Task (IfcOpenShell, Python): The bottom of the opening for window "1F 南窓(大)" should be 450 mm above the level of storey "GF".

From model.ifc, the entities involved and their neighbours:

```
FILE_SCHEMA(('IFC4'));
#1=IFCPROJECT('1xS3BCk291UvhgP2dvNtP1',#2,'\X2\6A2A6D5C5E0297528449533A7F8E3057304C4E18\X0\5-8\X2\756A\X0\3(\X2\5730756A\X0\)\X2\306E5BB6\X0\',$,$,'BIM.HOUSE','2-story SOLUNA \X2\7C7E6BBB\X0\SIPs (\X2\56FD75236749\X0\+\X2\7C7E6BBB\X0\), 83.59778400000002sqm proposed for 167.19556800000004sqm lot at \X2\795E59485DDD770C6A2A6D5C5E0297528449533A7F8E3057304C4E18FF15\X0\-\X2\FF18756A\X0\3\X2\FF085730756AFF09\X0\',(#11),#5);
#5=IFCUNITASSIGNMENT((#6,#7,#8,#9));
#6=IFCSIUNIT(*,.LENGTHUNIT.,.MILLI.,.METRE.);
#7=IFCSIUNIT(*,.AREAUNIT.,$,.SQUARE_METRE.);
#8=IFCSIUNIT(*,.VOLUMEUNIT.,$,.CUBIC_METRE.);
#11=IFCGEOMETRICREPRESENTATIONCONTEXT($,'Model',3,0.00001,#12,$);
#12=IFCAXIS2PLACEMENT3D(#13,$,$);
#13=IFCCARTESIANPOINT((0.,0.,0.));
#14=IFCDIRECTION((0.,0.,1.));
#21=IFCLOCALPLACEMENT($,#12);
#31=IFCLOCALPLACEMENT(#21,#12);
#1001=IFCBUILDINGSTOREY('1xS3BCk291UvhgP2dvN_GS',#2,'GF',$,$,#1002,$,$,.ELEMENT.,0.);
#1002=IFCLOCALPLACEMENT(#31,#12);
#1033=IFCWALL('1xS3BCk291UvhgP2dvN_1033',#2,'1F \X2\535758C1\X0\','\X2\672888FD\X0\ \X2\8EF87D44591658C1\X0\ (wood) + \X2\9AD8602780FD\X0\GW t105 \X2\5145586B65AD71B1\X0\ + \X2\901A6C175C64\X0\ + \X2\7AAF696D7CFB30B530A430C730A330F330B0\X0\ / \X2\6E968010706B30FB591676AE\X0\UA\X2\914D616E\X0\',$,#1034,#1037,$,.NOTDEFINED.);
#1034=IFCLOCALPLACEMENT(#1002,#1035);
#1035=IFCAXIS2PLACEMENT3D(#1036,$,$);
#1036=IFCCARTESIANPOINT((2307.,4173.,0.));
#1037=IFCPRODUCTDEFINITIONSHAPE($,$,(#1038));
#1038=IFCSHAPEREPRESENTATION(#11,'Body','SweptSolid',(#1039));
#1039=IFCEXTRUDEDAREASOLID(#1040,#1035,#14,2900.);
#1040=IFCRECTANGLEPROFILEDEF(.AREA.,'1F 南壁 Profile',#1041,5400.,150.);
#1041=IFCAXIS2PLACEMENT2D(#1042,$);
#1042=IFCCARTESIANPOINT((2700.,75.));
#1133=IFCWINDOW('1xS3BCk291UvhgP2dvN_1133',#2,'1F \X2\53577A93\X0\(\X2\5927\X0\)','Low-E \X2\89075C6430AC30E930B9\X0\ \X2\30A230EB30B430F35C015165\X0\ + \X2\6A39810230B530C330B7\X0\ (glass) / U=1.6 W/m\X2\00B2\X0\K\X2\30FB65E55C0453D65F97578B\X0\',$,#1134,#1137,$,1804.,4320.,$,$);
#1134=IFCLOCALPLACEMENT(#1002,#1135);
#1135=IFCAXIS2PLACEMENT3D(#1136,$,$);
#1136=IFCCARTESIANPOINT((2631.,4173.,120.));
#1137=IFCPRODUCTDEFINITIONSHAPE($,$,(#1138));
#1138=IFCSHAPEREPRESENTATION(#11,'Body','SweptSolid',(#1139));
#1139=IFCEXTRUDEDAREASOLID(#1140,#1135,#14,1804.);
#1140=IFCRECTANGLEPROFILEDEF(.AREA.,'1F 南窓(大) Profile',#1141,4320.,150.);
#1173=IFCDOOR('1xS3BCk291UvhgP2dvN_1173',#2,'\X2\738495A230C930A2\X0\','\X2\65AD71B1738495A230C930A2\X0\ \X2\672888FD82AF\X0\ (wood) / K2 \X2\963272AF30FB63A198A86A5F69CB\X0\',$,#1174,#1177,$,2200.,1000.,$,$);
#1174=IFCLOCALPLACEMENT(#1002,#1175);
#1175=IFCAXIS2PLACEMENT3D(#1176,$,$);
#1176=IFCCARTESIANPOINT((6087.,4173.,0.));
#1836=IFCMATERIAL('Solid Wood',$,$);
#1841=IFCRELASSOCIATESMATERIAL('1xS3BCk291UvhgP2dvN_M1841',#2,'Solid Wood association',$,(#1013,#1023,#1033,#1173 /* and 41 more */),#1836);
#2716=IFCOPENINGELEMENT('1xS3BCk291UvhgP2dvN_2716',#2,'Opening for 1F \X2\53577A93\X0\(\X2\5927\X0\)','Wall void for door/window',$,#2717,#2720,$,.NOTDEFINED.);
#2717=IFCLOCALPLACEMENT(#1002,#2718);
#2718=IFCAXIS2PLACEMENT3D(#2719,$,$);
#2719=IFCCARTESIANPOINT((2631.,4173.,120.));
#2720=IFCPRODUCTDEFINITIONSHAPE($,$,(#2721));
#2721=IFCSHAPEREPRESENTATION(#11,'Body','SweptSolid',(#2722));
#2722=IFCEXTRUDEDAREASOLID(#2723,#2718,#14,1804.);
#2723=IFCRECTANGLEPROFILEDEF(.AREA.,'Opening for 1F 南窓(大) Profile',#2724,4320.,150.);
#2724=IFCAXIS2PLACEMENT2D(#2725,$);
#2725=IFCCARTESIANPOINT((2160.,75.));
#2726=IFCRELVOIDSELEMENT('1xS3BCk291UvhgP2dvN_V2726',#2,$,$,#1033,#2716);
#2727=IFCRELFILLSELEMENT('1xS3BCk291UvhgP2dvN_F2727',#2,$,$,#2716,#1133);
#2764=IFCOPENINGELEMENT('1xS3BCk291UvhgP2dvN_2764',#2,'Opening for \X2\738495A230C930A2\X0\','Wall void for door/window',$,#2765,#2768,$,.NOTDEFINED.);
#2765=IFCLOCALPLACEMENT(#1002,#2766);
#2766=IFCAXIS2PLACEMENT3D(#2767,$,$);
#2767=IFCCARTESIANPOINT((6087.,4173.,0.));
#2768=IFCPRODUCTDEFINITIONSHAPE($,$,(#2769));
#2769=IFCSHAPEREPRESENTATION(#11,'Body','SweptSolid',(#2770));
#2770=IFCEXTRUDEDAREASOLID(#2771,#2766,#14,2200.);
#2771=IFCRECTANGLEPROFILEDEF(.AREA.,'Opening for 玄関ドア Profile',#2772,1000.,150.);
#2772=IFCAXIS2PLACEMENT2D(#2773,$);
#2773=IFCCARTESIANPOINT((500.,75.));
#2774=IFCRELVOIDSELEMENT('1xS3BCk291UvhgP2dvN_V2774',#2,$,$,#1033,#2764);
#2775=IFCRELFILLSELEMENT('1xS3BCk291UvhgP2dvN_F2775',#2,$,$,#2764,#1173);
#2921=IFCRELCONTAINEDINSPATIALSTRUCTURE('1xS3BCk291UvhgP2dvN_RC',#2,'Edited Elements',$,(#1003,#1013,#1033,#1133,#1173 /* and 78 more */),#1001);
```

```python
import numpy as np
import ifcopenshell
import ifcopenshell.api.geometry
import ifcopenshell.geom
import ifcopenshell.util.element
import ifcopenshell.util.placement
import ifcopenshell.util.shape
import ifcopenshell.util.unit

model = ifcopenshell.open("model.ifc")
unit_scale = ifcopenshell.util.unit.calculate_unit_scale(model)

window = model.by_guid("1xS3BCk291UvhgP2dvN_1133")
opening = window.FillsVoids[0].RelatingOpeningElement
storey = ifcopenshell.util.element.get_container(window, ifc_class="IfcBuildingStorey")
level = ifcopenshell.util.placement.get_local_placement(storey.ObjectPlacement)[2, 3]

# The opening's origin need not be at the sill, so measure its lowest point.
shape = ifcopenshell.geom.create_shape(ifcopenshell.geom.settings(), opening)
bottom = ifcopenshell.util.shape.get_shape_bottom_elevation(shape, shape.geometry) / unit_scale
dz = level + 0.45 / unit_scale - bottom

shift = np.array([0.0, 0.0, dz])
# The window is not placed relative to its opening, so move both.
for product in (opening, window):
    matrix = ifcopenshell.util.placement.get_local_placement(product.ObjectPlacement)
    matrix[:3, 3] += shift
    ifcopenshell.api.geometry.edit_object_placement(model, product=product, matrix=matrix, is_si=False)

print(f"moved by {dz * unit_scale:+.3f} m")

model.write("model_rev.ifc")
```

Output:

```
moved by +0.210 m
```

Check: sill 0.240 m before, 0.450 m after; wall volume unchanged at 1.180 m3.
